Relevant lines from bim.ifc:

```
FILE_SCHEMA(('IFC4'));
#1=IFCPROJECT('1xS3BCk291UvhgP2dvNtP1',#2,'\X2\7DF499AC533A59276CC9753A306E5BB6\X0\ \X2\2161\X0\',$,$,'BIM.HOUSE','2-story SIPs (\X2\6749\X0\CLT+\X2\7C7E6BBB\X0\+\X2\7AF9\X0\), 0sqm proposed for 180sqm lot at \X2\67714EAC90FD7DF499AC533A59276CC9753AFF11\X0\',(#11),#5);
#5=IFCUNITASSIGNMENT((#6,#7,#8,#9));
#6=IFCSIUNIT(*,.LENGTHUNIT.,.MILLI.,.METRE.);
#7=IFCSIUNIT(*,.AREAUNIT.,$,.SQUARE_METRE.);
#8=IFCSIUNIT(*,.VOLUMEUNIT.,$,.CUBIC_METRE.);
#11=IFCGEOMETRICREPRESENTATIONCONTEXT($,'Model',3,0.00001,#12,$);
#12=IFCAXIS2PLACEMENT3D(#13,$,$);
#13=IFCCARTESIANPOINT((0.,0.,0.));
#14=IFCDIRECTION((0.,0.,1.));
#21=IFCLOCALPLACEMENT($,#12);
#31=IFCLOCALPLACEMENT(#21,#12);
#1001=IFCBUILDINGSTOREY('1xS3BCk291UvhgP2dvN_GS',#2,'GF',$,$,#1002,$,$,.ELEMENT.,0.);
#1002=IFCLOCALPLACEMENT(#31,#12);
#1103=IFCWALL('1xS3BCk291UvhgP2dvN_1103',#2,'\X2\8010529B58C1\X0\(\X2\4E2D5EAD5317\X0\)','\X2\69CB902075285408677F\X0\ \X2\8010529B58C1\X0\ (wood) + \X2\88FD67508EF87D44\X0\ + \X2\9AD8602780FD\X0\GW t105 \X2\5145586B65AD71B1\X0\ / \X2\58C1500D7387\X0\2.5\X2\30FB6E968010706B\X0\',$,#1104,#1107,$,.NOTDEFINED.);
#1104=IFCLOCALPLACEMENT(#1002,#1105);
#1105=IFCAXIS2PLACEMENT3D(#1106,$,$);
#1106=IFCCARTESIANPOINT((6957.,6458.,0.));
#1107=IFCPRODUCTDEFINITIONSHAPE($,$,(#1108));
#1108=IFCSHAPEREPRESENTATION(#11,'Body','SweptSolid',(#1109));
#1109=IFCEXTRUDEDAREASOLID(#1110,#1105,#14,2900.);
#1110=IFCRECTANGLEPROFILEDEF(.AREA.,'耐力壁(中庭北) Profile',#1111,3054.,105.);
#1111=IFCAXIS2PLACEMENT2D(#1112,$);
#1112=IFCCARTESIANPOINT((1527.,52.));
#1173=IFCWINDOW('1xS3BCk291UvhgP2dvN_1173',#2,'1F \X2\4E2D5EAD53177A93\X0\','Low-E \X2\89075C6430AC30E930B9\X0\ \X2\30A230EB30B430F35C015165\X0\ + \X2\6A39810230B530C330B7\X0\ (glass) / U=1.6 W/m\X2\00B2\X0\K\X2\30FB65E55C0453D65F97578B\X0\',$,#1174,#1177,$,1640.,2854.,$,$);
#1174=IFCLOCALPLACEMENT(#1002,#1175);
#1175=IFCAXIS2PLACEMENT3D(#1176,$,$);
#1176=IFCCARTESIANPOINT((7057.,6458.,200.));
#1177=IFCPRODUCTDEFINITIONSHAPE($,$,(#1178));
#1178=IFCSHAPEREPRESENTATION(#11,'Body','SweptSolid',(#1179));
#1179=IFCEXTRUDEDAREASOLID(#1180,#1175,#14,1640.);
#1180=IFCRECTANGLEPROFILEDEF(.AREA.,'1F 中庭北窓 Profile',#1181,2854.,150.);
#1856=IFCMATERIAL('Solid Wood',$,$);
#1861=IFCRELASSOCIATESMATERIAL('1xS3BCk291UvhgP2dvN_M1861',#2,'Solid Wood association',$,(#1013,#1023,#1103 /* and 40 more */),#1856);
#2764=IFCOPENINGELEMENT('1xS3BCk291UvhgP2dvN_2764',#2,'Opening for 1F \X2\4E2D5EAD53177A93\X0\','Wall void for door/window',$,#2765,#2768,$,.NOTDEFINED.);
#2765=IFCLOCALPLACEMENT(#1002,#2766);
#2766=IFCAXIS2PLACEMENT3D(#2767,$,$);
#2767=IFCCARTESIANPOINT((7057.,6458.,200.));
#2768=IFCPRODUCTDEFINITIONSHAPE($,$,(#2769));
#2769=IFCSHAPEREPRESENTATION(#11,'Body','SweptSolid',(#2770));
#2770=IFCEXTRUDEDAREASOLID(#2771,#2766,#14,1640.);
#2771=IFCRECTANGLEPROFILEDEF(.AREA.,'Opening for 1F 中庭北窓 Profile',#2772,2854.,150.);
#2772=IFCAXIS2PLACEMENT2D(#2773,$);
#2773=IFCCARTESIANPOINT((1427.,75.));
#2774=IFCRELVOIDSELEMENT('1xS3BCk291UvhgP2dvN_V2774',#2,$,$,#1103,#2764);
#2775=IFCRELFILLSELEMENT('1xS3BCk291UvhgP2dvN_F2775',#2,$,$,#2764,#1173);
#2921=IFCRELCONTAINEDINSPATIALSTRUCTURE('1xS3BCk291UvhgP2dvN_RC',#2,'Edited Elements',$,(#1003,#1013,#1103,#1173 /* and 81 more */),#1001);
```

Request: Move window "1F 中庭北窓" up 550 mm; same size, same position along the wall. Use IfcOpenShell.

```python
import numpy as np
import ifcopenshell
import ifcopenshell.api.geometry
import ifcopenshell.util.placement
import ifcopenshell.util.unit

model = ifcopenshell.open("bim.ifc")
unit_scale = ifcopenshell.util.unit.calculate_unit_scale(model)

window = model.by_guid("1xS3BCk291UvhgP2dvN_1173")
opening = window.FillsVoids[0].RelatingOpeningElement
dz = 0.55 / unit_scale

shift = np.array([0.0, 0.0, dz])
# The window is not placed relative to its opening, so move both.
for product in (opening, window):
    matrix = ifcopenshell.util.placement.get_local_placement(product.ObjectPlacement)
    matrix[:3, 3] += shift
    ifcopenshell.api.geometry.edit_object_placement(model, product=product, matrix=matrix, is_si=False)

print(f"moved by {dz * unit_scale:+.3f} m")

model.write("bim_v2.ifc")
```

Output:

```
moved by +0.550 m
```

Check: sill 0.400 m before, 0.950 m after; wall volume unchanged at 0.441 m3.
